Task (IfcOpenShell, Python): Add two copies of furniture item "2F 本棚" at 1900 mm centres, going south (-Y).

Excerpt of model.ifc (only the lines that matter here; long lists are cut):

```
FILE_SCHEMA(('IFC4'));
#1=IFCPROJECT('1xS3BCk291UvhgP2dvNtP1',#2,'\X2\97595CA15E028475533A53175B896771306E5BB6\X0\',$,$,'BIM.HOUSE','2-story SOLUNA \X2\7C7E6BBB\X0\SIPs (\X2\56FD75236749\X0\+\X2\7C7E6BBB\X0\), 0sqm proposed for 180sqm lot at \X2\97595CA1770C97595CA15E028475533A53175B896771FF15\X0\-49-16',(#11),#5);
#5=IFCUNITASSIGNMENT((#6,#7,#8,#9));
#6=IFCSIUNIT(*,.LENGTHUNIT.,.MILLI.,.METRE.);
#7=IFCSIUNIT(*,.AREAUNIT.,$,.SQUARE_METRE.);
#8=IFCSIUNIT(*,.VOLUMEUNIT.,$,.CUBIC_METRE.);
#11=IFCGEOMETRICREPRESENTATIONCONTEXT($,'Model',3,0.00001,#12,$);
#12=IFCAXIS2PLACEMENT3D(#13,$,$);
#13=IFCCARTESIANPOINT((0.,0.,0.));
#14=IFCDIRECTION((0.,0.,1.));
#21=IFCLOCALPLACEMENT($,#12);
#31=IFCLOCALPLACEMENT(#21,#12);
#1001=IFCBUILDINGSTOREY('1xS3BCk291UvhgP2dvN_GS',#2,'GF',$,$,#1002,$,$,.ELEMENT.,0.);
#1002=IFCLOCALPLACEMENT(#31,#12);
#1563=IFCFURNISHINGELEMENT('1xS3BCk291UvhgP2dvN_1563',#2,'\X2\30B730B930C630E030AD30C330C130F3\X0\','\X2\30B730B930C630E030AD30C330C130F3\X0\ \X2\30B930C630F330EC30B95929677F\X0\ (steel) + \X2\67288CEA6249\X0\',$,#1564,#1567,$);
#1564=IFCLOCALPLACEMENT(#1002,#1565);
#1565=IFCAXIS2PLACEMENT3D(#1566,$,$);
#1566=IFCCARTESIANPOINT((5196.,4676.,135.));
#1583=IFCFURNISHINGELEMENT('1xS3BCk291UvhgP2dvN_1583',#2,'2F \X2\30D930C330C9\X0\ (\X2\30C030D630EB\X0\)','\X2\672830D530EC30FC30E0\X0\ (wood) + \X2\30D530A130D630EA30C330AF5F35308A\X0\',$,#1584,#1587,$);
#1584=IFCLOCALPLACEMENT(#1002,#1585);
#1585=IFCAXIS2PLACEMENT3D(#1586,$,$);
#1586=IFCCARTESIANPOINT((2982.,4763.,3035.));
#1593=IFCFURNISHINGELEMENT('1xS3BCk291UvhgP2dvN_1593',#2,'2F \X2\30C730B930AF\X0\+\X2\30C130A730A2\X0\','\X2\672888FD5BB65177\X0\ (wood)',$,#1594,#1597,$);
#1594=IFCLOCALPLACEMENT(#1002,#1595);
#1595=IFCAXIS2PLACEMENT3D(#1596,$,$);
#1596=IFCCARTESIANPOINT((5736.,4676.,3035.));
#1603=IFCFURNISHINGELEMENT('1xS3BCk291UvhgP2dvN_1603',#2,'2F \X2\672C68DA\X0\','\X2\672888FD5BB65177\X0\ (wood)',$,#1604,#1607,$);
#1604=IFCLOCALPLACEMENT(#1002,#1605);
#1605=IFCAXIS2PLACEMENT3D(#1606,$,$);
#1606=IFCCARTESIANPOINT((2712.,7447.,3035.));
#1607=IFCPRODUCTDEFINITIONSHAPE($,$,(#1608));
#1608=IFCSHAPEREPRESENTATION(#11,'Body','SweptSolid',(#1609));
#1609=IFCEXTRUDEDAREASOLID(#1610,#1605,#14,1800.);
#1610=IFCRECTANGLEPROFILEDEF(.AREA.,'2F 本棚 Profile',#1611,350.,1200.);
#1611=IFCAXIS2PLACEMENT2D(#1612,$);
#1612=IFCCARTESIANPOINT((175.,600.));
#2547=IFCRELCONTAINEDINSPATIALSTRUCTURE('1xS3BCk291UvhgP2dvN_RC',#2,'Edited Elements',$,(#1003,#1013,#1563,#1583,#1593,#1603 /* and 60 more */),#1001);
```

```python
import numpy as np
import ifcopenshell
import ifcopenshell.api.geometry
import ifcopenshell.api.root
import ifcopenshell.util.element
import ifcopenshell.util.placement

model = ifcopenshell.open("model.ifc")


def reuse_history(source, copy):
    """copy_class also copies each property set's owner history, people and application; keep the originals."""
    for rel in copy.IsDefinedBy:
        if rel.is_a("IfcRelDefinesByProperties") and (history := rel.RelatingPropertyDefinition.OwnerHistory):
            rel.RelatingPropertyDefinition.OwnerHistory = source.OwnerHistory
            ifcopenshell.util.element.remove_deep2(model, history)


source = model.by_id(1603)
base = ifcopenshell.util.placement.get_local_placement(source.ObjectPlacement)
step = np.array([0.0, -1.0, 0.0]) * 1900.0

for i in range(1, 3):
    copy = ifcopenshell.api.root.copy_class(model, product=source)
    copy.Representation = ifcopenshell.util.element.copy_deep(
        model, source.Representation, exclude=["IfcGeometricRepresentationContext", "IfcRepresentationMap"]
    )
    reuse_history(source, copy)
    matrix = base.copy()
    matrix[:3, 3] += i * step
    print("added at", matrix[:3, 3].round(3) + 0.0)
    ifcopenshell.api.geometry.edit_object_placement(model, product=copy, matrix=matrix, is_si=False)

model.write("model_rev.ifc")
```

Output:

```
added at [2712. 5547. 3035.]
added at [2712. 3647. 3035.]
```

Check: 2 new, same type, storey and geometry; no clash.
